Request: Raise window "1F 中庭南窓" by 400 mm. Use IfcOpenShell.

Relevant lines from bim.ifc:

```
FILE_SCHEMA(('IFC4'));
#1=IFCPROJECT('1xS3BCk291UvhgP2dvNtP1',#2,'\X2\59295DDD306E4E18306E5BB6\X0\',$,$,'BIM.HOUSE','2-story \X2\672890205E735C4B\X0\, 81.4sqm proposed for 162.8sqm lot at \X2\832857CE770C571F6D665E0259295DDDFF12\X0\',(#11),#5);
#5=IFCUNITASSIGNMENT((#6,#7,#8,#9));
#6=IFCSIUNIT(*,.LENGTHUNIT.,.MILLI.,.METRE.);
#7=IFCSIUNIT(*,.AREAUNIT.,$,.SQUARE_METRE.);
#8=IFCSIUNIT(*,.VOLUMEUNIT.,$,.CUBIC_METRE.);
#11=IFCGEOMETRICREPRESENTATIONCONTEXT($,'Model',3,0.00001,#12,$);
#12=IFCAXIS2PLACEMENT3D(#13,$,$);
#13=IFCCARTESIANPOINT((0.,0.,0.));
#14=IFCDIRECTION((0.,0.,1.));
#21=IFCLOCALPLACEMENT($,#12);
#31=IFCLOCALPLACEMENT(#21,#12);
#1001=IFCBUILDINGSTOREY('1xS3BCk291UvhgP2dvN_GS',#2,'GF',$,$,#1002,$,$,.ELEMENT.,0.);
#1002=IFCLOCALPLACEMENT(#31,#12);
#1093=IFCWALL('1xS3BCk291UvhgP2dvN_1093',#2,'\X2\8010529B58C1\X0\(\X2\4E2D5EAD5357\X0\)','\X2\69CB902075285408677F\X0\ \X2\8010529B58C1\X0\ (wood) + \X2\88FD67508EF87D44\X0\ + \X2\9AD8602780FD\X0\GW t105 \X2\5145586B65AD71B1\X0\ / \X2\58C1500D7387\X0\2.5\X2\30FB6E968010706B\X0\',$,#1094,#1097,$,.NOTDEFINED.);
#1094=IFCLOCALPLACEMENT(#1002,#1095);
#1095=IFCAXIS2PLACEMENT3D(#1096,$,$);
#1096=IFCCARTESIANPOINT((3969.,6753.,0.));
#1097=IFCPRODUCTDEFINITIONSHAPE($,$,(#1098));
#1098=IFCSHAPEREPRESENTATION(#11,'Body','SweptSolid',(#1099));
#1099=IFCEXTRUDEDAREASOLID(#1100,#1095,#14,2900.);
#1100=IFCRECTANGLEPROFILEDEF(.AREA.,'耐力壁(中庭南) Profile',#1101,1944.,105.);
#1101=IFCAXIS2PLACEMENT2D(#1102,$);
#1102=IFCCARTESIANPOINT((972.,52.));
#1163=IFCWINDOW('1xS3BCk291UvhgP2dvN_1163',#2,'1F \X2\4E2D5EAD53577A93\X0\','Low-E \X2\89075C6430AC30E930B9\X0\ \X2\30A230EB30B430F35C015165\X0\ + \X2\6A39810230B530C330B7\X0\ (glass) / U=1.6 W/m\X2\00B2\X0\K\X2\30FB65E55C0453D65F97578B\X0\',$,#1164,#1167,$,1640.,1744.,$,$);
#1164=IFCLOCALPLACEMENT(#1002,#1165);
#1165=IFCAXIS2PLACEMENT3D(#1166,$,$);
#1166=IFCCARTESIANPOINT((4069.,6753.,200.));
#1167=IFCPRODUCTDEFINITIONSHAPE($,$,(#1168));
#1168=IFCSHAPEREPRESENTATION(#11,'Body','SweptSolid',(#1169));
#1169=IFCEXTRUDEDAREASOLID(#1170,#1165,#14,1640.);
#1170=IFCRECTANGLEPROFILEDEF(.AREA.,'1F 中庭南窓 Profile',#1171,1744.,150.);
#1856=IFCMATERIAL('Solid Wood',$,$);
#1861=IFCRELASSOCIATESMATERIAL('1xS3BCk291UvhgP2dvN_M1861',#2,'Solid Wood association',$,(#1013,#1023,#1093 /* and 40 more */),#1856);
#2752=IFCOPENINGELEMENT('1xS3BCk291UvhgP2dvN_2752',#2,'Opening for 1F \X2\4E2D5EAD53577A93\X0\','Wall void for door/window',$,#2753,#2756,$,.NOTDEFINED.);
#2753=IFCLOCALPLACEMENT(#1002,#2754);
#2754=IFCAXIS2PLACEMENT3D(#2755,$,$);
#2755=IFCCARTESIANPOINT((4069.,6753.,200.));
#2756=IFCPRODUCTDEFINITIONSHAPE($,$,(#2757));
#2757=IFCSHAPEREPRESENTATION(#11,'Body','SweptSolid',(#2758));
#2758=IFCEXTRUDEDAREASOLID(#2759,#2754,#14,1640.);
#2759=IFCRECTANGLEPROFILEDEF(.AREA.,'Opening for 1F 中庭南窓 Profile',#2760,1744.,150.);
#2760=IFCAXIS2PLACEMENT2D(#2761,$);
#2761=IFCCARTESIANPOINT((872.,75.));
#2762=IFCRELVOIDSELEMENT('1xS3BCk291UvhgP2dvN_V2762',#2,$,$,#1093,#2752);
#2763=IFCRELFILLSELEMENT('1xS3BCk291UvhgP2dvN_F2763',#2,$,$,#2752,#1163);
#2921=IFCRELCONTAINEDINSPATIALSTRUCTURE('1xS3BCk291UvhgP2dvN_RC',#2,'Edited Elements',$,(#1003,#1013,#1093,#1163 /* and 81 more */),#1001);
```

```python
import numpy as np
import ifcopenshell
import ifcopenshell.api.geometry
import ifcopenshell.util.placement
import ifcopenshell.util.unit

model = ifcopenshell.open("bim.ifc")
unit_scale = ifcopenshell.util.unit.calculate_unit_scale(model)

window = model.by_guid("1xS3BCk291UvhgP2dvN_1163")
opening = window.FillsVoids[0].RelatingOpeningElement
dz = 0.4 / unit_scale

shift = np.array([0.0, 0.0, dz])
# The window is not placed relative to its opening, so move both.
for product in (opening, window):
    matrix = ifcopenshell.util.placement.get_local_placement(product.ObjectPlacement)
    matrix[:3, 3] += shift
    ifcopenshell.api.geometry.edit_object_placement(model, product=product, matrix=matrix, is_si=False)

print(f"moved by {dz * unit_scale:+.3f} m")

model.write("bim-out.ifc")
```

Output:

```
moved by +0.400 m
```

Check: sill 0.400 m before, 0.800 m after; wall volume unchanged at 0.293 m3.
